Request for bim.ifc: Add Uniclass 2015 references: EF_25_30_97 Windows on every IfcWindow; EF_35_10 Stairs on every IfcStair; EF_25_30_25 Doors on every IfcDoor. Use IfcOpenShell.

First a look at what the model holds.

```python
import ifcopenshell

model = ifcopenshell.open("bim.ifc")
print(model.schema)
print("classifications:", [c.Name for c in model.by_type("IfcClassification")])
for ifc_class in ("IfcDoor", "IfcRoof", "IfcStair", "IfcWall", "IfcWindow"):
    print(ifc_class, len(model.by_type(ifc_class)))
```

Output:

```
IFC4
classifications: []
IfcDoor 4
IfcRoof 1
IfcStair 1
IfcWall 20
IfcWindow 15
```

```python
import ifcopenshell
import ifcopenshell.api.classification

model = ifcopenshell.open("bim.ifc")

system = ifcopenshell.api.classification.add_classification(model, classification="Uniclass 2015")

codes = {
    "IfcWindow": ("EF_25_30_97", "Windows"),
    "IfcStair": ("EF_35_10", "Stairs"),
    "IfcDoor": ("EF_25_30_25", "Doors"),
}
for ifc_class, (code, name) in codes.items():
    products = model.by_type(ifc_class)
    ifcopenshell.api.classification.add_reference(
        model, products=products, classification=system, identification=code, name=name
    )
    print(code, len(products))

model.write("bim_updated.ifc")
```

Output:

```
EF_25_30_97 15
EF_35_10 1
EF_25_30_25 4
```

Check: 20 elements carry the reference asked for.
